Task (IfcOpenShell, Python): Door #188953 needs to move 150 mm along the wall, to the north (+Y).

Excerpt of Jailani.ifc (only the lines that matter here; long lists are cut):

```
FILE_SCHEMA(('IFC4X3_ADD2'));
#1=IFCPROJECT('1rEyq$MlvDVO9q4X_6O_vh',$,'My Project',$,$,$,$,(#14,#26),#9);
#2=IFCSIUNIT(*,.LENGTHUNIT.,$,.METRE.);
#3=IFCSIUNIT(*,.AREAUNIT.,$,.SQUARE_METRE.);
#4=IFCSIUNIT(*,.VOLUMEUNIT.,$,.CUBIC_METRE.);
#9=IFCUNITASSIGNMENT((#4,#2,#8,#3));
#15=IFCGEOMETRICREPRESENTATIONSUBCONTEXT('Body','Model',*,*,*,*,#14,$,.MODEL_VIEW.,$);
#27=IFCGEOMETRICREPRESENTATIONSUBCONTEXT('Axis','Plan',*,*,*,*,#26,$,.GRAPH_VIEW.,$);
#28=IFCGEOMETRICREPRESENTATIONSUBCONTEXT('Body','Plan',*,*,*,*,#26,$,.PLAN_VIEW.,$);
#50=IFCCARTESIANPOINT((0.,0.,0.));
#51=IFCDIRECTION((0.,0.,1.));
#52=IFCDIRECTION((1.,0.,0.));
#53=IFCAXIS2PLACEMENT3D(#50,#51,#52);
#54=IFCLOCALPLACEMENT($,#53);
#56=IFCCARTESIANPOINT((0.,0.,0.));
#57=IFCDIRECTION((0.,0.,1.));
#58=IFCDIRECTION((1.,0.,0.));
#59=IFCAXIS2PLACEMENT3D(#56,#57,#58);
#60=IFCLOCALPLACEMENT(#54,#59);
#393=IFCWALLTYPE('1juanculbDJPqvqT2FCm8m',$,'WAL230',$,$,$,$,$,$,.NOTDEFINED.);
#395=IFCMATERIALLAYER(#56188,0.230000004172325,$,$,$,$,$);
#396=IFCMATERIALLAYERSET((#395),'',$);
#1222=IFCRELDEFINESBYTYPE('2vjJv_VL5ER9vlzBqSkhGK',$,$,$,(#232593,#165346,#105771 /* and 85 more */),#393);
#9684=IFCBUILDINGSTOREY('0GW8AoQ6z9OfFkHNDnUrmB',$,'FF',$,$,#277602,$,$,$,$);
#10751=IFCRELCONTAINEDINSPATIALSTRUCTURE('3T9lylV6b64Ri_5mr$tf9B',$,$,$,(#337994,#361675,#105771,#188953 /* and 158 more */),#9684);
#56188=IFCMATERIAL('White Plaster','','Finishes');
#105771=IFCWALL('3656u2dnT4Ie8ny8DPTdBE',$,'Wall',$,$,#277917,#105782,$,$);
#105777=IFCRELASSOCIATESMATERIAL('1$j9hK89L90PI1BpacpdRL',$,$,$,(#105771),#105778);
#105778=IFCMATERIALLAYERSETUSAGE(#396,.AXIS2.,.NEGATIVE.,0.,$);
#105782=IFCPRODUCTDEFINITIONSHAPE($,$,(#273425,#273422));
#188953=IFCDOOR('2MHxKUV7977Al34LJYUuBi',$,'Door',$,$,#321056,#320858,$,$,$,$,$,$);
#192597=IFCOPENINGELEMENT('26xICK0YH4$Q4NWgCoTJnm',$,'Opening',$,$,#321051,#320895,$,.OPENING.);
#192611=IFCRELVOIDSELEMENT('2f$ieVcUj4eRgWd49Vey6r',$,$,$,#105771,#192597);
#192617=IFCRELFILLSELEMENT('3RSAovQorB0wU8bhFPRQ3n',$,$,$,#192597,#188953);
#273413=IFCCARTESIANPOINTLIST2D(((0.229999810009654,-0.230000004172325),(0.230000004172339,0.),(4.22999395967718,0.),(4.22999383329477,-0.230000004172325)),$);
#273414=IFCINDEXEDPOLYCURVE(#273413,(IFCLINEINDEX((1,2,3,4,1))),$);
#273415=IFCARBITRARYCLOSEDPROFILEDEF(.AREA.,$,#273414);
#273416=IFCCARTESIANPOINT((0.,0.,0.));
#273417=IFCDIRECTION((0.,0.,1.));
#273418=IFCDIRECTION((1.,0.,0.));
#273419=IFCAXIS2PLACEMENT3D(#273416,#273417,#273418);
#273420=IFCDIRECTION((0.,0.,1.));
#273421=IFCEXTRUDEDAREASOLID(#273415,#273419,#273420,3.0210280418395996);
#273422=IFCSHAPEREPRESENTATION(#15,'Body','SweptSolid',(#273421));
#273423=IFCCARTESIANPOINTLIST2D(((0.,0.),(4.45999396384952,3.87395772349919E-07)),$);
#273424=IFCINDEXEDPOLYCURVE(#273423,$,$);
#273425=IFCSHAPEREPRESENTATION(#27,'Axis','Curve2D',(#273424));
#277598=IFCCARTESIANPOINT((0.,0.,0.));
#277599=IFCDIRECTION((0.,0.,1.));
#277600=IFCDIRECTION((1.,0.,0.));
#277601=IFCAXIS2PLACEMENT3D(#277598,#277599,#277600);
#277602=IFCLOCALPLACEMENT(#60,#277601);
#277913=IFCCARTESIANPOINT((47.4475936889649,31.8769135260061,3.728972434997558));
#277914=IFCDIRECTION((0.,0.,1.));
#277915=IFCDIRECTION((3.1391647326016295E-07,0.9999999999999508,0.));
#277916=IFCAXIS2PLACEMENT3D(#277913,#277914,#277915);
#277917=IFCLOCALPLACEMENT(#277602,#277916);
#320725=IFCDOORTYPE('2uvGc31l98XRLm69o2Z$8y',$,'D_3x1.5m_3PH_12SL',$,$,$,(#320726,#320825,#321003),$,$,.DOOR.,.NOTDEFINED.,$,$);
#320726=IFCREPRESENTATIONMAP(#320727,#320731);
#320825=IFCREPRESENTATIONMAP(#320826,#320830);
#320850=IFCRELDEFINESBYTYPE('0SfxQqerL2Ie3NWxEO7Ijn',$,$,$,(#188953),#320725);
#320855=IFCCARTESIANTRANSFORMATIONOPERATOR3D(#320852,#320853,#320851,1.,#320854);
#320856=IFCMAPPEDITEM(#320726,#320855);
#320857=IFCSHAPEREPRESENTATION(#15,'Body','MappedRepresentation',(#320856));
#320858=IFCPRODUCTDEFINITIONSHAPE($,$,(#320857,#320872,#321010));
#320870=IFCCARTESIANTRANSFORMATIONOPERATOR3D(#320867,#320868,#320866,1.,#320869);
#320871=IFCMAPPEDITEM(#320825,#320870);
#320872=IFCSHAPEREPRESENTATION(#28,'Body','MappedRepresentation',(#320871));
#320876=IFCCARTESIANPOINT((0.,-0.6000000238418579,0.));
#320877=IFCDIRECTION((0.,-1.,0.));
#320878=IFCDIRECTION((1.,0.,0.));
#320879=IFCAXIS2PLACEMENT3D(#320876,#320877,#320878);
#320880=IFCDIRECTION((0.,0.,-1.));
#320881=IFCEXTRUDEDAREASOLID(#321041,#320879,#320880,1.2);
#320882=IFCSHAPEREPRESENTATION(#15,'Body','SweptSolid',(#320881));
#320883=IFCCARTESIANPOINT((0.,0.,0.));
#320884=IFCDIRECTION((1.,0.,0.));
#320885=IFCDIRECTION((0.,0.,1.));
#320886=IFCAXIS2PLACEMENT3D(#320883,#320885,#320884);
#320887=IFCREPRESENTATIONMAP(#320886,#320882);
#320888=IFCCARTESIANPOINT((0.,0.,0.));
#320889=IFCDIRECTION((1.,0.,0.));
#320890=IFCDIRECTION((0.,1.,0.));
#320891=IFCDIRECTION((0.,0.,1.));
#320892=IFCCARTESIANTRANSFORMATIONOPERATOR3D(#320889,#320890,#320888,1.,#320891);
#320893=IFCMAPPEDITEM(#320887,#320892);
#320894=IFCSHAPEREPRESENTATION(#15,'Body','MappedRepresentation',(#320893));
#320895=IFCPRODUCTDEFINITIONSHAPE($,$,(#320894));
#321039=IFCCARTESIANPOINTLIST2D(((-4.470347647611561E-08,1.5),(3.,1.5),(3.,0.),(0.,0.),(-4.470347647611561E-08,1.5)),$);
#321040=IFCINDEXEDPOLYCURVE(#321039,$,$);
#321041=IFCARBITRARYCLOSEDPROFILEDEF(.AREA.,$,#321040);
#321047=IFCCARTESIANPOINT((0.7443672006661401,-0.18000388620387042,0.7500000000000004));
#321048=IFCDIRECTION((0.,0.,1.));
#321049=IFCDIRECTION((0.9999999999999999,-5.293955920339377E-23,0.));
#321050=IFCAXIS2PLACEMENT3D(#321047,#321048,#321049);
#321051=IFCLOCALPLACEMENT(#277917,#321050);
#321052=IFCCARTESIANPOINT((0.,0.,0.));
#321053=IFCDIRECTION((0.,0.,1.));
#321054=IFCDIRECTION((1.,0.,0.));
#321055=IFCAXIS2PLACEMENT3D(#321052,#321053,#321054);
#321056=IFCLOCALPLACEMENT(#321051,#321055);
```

```python
import ifcopenshell
import ifcopenshell.api.geometry
import ifcopenshell.util.placement
import ifcopenshell.util.unit

model = ifcopenshell.open("Jailani.ifc")
unit_scale = ifcopenshell.util.unit.calculate_unit_scale(model)

door = model.by_guid("2MHxKUV7977Al34LJYUuBi")
opening = door.FillsVoids[0].RelatingOpeningElement
wall = opening.VoidsElements[0].RelatingBuildingElement

wall_matrix = ifcopenshell.util.placement.get_local_placement(wall.ObjectPlacement)
shift = wall_matrix[:3, 0] * 0.15 / unit_scale
before = ifcopenshell.util.placement.get_local_placement(door.ObjectPlacement)[:3, 3].copy()

# The door is placed relative to its opening, so it follows when the opening moves.
matrix = ifcopenshell.util.placement.get_local_placement(opening.ObjectPlacement)
matrix[:3, 3] += shift
ifcopenshell.api.geometry.edit_object_placement(
    model, product=opening, matrix=matrix, is_si=False, should_transform_children=True
)

after = ifcopenshell.util.placement.get_local_placement(door.ObjectPlacement)[:3, 3]
print("door moved by", (after - before).round(3) + 0.0)

model.write("Jailani-out.ifc")
```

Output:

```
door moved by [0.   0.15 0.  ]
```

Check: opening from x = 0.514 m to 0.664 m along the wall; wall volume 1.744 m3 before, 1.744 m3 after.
